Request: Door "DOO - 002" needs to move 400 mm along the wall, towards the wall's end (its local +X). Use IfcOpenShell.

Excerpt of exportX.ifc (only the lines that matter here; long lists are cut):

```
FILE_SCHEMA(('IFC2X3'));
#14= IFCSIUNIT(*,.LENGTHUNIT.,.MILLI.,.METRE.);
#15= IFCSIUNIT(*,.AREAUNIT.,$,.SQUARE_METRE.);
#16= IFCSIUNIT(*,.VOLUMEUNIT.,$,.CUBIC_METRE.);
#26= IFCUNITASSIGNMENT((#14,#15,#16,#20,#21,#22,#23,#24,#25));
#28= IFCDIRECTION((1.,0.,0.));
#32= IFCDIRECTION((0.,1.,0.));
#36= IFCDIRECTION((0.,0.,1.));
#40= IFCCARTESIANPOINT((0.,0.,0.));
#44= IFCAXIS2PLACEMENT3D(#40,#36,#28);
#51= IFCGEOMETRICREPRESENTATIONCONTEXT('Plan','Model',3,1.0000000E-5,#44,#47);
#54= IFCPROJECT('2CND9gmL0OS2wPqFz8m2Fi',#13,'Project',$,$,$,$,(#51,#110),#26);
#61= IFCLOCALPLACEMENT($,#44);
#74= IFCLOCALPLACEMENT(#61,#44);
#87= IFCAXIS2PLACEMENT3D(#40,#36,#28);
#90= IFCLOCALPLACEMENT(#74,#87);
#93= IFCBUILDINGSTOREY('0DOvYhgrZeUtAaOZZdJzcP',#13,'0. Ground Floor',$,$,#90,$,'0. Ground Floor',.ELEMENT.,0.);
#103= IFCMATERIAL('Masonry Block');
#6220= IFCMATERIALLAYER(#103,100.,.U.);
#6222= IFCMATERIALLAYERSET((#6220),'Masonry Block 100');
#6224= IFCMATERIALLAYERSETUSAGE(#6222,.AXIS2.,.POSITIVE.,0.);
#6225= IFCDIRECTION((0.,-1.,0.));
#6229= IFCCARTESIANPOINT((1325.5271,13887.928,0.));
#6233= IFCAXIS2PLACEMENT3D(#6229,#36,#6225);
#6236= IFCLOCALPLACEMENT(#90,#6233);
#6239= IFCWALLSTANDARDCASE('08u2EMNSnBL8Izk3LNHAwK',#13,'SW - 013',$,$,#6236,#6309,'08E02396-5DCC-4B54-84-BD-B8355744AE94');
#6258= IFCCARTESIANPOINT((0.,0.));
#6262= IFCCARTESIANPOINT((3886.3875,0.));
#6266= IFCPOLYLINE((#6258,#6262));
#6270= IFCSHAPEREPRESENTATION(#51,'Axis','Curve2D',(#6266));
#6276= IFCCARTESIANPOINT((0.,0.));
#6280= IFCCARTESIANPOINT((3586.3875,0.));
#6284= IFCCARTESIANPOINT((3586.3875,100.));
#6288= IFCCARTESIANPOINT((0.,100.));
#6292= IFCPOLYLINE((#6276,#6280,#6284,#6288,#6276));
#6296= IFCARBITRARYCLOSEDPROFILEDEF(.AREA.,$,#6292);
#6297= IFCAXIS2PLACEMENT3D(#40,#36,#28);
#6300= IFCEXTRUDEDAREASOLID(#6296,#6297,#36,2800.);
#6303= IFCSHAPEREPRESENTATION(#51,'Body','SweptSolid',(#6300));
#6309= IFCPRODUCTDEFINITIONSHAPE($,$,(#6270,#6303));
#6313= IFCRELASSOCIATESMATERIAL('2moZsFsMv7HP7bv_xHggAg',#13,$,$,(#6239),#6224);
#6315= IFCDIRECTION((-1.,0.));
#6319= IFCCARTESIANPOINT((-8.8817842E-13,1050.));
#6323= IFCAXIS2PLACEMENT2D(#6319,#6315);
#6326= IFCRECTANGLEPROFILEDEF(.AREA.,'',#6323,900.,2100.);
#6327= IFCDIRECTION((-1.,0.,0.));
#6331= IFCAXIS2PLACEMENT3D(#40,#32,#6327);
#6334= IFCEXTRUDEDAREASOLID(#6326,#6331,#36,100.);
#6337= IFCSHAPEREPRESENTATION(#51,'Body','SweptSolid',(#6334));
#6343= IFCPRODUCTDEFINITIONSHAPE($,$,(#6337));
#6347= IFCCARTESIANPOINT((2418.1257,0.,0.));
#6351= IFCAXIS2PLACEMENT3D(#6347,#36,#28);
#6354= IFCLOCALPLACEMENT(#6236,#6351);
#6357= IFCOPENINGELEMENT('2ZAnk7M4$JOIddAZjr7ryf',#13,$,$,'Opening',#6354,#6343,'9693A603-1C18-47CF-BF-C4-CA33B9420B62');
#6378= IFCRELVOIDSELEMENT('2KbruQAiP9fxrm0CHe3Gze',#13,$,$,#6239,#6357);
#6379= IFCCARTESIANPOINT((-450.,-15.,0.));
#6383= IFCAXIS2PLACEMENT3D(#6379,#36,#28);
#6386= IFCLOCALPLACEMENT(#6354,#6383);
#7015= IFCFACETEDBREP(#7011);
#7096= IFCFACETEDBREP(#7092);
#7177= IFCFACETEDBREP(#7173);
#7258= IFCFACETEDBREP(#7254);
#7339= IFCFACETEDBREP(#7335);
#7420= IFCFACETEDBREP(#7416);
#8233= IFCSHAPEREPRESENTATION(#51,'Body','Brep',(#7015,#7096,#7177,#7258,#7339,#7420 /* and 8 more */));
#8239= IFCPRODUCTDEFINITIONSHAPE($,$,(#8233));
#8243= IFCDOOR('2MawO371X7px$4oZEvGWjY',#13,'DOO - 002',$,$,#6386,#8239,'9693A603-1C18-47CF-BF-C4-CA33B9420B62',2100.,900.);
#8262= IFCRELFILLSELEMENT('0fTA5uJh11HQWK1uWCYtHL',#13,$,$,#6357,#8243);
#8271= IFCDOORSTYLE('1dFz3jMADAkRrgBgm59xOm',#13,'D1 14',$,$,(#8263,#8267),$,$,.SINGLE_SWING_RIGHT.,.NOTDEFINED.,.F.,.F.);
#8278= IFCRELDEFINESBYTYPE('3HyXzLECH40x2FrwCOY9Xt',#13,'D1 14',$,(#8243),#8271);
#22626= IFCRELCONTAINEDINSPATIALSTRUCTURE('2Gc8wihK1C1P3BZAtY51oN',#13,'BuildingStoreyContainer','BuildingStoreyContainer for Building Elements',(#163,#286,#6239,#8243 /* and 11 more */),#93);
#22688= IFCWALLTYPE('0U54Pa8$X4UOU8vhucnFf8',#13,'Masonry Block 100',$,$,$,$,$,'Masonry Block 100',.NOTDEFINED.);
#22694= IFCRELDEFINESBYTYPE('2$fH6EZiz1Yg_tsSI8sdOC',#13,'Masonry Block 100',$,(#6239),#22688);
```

```python
import ifcopenshell
import ifcopenshell.api.geometry
import ifcopenshell.util.placement
import ifcopenshell.util.unit

model = ifcopenshell.open("exportX.ifc")
unit_scale = ifcopenshell.util.unit.calculate_unit_scale(model)

door = model.by_guid("2MawO371X7px$4oZEvGWjY")
opening = door.FillsVoids[0].RelatingOpeningElement
wall = opening.VoidsElements[0].RelatingBuildingElement

wall_matrix = ifcopenshell.util.placement.get_local_placement(wall.ObjectPlacement)
shift = wall_matrix[:3, 0] * 0.4 / unit_scale
before = ifcopenshell.util.placement.get_local_placement(door.ObjectPlacement)[:3, 3].copy()

# The door is placed relative to its opening, so it follows when the opening moves.
matrix = ifcopenshell.util.placement.get_local_placement(opening.ObjectPlacement)
matrix[:3, 3] += shift
ifcopenshell.api.geometry.edit_object_placement(
    model, product=opening, matrix=matrix, is_si=False, should_transform_children=True
)

after = ifcopenshell.util.placement.get_local_placement(door.ObjectPlacement)[:3, 3]
print("door moved by", (after - before).round(3) + 0.0)

model.write("exportX_updated.ifc")
```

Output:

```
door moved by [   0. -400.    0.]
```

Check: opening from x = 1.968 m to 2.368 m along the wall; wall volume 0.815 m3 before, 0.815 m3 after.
